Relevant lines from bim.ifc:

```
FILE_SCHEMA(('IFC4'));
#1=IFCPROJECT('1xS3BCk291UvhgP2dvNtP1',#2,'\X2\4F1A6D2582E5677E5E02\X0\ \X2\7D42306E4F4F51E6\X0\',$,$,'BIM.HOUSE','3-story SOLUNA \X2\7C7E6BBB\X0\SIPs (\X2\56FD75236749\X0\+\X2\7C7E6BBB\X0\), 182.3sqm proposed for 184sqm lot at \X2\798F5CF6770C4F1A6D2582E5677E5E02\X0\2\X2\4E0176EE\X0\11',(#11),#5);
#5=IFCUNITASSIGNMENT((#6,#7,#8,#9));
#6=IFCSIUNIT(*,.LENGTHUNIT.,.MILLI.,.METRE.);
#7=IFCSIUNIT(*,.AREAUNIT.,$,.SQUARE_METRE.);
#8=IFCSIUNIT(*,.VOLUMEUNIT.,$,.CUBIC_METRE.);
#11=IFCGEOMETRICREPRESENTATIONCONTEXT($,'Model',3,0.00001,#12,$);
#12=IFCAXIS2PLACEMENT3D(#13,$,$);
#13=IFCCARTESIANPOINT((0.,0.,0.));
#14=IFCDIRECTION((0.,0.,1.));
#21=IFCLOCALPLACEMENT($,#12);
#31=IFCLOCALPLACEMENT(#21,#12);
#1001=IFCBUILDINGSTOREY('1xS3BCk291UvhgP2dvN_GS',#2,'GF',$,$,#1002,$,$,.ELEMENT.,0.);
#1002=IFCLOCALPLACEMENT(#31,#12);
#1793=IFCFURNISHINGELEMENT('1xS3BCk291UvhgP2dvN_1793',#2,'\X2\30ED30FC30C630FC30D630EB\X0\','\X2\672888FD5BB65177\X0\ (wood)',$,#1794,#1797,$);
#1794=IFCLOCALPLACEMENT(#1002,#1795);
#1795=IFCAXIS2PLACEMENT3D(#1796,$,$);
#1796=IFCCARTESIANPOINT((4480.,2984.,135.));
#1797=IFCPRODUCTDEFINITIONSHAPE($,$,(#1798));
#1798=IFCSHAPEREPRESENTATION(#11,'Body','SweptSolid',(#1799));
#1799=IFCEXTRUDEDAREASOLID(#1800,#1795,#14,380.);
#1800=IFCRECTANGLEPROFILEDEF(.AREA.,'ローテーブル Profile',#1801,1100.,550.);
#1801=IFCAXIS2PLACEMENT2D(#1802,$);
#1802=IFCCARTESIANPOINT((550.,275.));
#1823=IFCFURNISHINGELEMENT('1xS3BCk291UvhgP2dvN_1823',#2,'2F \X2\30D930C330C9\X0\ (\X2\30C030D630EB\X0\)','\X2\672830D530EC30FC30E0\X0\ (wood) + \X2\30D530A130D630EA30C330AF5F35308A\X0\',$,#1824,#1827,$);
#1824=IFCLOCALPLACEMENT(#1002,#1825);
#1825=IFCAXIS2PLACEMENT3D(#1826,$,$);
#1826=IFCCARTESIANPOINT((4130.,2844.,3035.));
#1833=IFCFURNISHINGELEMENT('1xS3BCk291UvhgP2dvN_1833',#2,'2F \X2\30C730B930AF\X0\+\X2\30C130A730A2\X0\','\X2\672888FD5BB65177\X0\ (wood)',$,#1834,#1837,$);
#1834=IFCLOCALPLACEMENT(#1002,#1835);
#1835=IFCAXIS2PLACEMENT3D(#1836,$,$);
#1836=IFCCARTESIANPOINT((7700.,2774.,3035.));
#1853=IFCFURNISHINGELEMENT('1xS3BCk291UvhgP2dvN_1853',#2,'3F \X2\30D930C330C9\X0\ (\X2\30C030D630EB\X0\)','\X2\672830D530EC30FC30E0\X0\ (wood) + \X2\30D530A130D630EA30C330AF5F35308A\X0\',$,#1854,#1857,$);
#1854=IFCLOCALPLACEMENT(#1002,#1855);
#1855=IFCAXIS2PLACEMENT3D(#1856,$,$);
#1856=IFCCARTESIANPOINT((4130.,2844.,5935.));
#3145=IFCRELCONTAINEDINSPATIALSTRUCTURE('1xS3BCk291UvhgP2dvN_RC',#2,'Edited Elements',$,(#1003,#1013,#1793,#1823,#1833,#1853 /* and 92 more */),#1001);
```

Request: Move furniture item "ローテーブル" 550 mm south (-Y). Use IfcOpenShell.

```python
import ifcopenshell
import ifcopenshell.api.geometry
import ifcopenshell.util.placement
import ifcopenshell.util.unit

model = ifcopenshell.open("bim.ifc")
unit_scale = ifcopenshell.util.unit.calculate_unit_scale(model)

item = model.by_id(1793)
matrix = ifcopenshell.util.placement.get_local_placement(item.ObjectPlacement)
matrix[1, 3] -= 0.55 / unit_scale
ifcopenshell.api.geometry.edit_object_placement(model, product=item, matrix=matrix, is_si=False)

print(ifcopenshell.util.placement.get_local_placement(item.ObjectPlacement).round(3) + 0.0)

model.write("bim_updated.ifc")
```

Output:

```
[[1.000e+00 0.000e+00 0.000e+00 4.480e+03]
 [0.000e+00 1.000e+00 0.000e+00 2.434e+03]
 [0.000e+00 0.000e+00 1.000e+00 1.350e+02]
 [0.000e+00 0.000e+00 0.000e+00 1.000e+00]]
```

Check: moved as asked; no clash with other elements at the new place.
